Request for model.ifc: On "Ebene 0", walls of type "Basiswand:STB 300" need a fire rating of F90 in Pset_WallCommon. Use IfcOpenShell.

First a look at what the model holds.

```python
import ifcopenshell
import ifcopenshell.util.element

model = ifcopenshell.open("model.ifc")
print(model.schema)
storey = next(s for s in model.by_type("IfcBuildingStorey") if s.Name == "Ebene 0")
walls = [e for e in ifcopenshell.util.element.get_decomposition(storey) if e.is_a("IfcWall")]
seen = {}
for e in walls:
    element_type = ifcopenshell.util.element.get_type(e)
    key = (element_type.Name if element_type != e and element_type else None, ifcopenshell.util.element.get_pset(e, "Pset_WallCommon", "FireRating"))
    seen[key] = seen.get(key, 0) + 1
for (name, value), count in sorted(seen.items(), key=str):
    print(count, "x", name, "|", value)
```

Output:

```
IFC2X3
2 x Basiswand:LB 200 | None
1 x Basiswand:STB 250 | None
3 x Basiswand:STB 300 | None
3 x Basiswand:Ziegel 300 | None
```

```python
import ifcopenshell
import ifcopenshell.api.pset
import ifcopenshell.util.element

model = ifcopenshell.open("model.ifc")

storey = next(s for s in model.by_type("IfcBuildingStorey") if s.Name == "Ebene 0")
walls = [e for e in ifcopenshell.util.element.get_decomposition(storey) if e.is_a("IfcWall")]

count = 0
for e in walls:
    element_type = ifcopenshell.util.element.get_type(e)
    if element_type in (None, e) or element_type.Name != "Basiswand:STB 300":
        continue
    # add_pset returns the element's existing set when there is one.
    pset = ifcopenshell.api.pset.add_pset(model, product=e, name="Pset_WallCommon")
    ifcopenshell.api.pset.edit_pset(model, pset=pset, properties={"FireRating": "F90"})
    count += 1

print(count, "walls updated")

model.write("model_edited.ifc")
```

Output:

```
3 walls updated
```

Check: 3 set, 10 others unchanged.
